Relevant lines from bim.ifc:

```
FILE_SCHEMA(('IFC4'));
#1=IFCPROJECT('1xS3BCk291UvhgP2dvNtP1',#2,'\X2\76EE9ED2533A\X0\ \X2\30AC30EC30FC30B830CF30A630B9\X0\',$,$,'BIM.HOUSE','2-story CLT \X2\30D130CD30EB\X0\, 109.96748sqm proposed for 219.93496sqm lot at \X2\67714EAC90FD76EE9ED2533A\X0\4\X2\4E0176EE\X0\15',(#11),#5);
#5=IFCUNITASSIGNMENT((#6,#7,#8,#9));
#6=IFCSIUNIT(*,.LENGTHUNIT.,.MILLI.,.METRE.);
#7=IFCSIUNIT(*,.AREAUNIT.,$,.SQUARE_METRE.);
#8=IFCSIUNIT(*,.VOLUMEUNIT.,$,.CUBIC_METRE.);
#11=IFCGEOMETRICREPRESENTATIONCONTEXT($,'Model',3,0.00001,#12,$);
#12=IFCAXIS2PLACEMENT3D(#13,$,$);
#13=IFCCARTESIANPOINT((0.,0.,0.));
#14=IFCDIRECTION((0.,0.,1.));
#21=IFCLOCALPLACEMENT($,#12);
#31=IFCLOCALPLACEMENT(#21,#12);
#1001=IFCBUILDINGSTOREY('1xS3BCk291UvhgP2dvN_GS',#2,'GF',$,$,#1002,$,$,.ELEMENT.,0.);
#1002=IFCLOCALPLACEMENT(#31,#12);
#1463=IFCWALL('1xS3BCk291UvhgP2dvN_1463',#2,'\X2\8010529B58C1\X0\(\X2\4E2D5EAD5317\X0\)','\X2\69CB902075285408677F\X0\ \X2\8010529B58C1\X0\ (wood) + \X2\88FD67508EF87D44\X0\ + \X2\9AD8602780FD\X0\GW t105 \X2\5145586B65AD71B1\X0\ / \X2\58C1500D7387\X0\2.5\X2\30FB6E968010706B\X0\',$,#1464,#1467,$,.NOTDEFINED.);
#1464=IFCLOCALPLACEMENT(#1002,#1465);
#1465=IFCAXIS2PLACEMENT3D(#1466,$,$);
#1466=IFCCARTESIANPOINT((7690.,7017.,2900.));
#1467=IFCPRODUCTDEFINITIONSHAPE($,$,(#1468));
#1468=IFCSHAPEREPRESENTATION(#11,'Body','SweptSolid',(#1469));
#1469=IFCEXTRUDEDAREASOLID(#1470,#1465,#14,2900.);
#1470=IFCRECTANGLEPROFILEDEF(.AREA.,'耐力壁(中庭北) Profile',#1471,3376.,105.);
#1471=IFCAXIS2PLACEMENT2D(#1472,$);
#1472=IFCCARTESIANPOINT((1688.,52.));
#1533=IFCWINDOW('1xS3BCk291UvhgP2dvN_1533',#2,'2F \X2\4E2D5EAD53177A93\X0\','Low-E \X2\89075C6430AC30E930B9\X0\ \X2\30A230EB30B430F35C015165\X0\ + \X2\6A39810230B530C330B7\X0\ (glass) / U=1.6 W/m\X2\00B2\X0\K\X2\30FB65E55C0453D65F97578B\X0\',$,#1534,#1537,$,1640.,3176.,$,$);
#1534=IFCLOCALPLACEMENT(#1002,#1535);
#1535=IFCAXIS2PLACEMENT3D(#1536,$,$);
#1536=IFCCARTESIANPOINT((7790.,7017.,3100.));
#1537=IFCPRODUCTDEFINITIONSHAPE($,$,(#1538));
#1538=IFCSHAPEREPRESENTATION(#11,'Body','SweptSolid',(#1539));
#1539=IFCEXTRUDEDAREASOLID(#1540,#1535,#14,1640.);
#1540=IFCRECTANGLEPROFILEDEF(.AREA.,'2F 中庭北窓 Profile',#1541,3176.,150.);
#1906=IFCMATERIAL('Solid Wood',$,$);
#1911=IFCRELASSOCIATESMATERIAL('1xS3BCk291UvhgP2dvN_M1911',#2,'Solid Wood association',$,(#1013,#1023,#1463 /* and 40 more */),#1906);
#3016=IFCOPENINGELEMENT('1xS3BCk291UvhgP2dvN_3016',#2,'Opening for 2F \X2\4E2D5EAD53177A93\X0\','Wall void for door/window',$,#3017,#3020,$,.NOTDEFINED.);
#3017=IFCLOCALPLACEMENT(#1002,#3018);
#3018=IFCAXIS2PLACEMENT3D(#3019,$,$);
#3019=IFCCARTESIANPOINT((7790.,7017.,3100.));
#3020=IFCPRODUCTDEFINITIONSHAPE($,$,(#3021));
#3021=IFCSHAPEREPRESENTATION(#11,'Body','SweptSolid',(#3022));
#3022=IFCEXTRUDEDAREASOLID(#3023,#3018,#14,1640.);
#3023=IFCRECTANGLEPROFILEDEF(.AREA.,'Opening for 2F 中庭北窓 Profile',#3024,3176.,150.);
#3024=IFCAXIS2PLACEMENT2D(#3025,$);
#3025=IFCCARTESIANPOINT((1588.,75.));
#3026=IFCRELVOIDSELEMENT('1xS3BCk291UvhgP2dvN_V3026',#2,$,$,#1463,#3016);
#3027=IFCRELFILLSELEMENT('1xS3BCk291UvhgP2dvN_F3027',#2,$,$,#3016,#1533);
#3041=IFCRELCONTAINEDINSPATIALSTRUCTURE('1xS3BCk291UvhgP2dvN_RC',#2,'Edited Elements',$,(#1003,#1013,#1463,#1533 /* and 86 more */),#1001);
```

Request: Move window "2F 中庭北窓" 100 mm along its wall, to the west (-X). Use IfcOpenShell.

```python
import ifcopenshell
import ifcopenshell.api.geometry
import ifcopenshell.util.placement
import ifcopenshell.util.unit

model = ifcopenshell.open("bim.ifc")
unit_scale = ifcopenshell.util.unit.calculate_unit_scale(model)

window = model.by_guid("1xS3BCk291UvhgP2dvN_1533")
opening = window.FillsVoids[0].RelatingOpeningElement
wall = opening.VoidsElements[0].RelatingBuildingElement

wall_matrix = ifcopenshell.util.placement.get_local_placement(wall.ObjectPlacement)
shift = wall_matrix[:3, 0] * -0.1 / unit_scale
before = ifcopenshell.util.placement.get_local_placement(window.ObjectPlacement)[:3, 3].copy()

# The window is not placed relative to its opening, so move both.
for product in (opening, window):
    matrix = ifcopenshell.util.placement.get_local_placement(product.ObjectPlacement)
    matrix[:3, 3] += shift
    ifcopenshell.api.geometry.edit_object_placement(model, product=product, matrix=matrix, is_si=False)

after = ifcopenshell.util.placement.get_local_placement(window.ObjectPlacement)[:3, 3]
print("window moved by", (after - before).round(3) + 0.0)

model.write("bim_edited.ifc")
```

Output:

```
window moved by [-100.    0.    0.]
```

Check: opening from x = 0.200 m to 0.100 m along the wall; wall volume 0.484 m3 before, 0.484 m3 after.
